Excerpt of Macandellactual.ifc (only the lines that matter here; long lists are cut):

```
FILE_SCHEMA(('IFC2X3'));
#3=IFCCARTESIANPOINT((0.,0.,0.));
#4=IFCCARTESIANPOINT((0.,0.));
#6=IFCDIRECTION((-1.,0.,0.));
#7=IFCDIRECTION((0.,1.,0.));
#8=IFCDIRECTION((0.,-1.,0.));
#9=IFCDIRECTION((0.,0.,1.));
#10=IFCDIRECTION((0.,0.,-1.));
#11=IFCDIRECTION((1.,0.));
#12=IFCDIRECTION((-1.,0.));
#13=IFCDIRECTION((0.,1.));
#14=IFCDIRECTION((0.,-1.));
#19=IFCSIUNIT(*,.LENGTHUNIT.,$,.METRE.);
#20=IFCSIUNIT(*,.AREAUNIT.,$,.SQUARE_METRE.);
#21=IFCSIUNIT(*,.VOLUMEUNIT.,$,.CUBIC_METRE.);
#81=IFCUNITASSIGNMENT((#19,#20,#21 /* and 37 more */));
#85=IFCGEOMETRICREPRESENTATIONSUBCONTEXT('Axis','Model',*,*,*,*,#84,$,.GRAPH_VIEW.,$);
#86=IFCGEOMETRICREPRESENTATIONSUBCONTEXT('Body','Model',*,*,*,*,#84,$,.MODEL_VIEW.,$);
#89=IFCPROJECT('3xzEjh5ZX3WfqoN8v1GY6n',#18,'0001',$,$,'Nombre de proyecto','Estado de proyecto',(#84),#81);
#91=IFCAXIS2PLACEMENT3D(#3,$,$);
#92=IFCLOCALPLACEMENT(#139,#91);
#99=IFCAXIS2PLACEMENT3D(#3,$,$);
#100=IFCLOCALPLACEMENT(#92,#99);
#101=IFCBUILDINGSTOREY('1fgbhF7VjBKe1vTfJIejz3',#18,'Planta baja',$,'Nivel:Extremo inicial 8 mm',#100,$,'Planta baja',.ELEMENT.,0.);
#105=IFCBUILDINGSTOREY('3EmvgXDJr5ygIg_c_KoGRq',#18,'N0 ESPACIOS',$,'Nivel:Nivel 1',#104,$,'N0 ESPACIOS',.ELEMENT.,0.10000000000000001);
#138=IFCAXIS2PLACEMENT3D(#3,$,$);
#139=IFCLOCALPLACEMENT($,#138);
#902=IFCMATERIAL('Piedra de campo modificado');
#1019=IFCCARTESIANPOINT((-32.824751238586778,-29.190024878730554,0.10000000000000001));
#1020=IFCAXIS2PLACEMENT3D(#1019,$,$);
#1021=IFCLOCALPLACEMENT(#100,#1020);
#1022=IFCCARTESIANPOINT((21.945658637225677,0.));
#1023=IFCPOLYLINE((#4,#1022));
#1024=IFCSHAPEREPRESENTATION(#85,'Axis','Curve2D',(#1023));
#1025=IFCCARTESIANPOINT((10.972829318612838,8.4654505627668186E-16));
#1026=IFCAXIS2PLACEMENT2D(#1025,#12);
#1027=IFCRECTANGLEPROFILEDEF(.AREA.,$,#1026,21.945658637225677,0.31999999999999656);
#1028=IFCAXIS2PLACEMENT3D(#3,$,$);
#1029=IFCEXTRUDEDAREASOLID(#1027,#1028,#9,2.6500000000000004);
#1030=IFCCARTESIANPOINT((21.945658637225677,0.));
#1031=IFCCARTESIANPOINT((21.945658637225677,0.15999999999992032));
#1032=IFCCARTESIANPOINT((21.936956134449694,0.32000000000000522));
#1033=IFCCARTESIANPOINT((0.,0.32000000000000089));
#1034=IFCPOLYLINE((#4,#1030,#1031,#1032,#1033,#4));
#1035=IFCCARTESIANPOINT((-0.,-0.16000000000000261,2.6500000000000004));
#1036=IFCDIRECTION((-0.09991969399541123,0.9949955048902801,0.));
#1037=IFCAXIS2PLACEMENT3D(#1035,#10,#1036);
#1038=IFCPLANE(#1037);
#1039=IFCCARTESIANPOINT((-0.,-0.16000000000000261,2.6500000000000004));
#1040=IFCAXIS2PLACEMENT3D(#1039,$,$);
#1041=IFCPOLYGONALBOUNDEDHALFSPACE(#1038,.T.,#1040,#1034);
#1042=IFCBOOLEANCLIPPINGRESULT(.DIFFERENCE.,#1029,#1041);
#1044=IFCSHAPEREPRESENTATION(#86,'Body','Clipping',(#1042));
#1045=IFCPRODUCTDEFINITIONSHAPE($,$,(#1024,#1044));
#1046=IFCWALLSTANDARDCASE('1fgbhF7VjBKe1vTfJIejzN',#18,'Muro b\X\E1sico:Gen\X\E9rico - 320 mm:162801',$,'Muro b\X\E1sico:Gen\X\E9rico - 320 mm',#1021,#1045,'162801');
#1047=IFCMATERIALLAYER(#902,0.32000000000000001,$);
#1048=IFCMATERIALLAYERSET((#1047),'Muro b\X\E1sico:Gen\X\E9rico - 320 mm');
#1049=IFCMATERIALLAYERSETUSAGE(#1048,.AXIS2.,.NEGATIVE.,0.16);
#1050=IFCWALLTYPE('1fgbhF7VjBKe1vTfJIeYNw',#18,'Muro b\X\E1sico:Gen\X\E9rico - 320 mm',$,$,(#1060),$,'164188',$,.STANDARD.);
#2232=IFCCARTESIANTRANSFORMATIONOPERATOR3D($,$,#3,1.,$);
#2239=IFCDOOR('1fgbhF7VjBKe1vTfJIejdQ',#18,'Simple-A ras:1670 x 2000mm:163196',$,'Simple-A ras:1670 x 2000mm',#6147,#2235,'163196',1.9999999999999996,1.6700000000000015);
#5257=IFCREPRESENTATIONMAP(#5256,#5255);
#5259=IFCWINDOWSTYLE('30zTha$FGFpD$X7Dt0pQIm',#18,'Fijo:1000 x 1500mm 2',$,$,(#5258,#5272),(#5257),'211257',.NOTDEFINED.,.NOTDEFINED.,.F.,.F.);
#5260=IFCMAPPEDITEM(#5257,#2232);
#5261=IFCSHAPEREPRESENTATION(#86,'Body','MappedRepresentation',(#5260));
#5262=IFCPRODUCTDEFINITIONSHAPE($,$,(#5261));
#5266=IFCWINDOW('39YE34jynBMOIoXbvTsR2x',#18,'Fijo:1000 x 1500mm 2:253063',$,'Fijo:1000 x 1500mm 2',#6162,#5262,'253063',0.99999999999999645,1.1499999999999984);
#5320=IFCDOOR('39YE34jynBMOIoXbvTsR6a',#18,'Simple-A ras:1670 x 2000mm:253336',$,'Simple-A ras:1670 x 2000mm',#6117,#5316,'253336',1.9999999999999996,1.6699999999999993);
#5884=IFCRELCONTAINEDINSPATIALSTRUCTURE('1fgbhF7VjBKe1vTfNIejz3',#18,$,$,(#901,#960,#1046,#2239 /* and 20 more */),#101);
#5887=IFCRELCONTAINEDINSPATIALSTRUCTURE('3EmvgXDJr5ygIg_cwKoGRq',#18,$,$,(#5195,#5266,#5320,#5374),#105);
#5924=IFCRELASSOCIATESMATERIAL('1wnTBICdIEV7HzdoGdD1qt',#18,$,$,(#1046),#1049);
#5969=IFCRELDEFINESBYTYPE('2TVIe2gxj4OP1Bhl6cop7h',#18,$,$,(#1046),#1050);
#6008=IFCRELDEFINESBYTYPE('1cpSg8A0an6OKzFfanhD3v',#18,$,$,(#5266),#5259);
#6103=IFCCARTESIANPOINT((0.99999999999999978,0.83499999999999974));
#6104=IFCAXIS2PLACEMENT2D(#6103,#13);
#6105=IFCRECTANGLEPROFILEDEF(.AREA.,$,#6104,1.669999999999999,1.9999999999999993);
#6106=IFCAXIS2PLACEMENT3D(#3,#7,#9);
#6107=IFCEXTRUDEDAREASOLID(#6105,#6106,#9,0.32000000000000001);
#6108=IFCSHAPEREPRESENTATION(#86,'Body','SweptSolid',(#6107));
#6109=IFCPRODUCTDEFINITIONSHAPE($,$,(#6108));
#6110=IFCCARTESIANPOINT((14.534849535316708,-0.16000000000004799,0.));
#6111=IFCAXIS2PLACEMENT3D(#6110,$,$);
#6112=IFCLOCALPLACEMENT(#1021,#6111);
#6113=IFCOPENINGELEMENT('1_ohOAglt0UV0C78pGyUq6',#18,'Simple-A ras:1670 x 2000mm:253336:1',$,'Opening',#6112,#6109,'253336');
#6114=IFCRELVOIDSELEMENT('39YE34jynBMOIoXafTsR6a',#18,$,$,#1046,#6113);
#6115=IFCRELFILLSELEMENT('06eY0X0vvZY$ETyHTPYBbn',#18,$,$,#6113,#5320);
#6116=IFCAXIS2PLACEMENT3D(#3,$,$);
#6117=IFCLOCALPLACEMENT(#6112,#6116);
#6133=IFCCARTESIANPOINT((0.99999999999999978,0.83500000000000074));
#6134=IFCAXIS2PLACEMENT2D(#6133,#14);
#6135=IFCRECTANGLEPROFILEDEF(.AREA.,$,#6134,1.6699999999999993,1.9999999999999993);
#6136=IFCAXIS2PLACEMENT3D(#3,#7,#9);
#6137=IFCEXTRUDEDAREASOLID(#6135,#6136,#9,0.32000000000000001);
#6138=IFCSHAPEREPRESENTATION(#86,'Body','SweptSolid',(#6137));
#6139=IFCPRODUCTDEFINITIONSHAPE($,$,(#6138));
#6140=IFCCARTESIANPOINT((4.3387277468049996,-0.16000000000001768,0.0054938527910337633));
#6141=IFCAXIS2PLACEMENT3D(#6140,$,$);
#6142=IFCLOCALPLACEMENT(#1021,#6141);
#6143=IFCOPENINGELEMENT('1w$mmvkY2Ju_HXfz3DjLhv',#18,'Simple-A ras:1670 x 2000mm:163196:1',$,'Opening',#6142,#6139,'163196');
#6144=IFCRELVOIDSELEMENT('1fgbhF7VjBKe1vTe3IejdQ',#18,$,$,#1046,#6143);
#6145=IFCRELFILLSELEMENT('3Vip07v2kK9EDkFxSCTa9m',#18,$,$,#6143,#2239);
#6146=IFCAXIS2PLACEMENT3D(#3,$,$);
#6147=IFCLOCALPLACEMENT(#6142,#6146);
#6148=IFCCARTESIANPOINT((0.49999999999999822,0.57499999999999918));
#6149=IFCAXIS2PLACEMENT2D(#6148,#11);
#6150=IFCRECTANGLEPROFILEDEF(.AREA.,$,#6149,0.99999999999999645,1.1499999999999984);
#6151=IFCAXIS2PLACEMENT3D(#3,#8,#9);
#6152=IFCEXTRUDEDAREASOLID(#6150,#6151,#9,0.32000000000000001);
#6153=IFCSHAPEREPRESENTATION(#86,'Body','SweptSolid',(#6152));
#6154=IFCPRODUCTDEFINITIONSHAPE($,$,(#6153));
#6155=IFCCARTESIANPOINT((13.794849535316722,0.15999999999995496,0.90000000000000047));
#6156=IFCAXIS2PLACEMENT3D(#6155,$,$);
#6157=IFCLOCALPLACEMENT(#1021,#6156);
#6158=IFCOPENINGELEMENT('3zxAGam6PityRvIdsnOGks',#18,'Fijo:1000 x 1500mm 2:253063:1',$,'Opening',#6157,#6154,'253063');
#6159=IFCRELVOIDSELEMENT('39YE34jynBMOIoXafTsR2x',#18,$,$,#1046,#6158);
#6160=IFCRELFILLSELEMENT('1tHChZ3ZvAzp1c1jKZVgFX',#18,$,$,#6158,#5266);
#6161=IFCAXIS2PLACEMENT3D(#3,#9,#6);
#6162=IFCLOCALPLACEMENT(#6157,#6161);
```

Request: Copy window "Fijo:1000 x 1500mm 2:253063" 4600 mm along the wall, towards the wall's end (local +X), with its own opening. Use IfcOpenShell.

```python
import ifcopenshell
import ifcopenshell.api.feature
import ifcopenshell.api.geometry
import ifcopenshell.api.root
import ifcopenshell.geom
import ifcopenshell.util.element
import ifcopenshell.util.placement
import ifcopenshell.util.shape
import ifcopenshell.util.unit

model = ifcopenshell.open("Macandellactual.ifc")
unit_scale = ifcopenshell.util.unit.calculate_unit_scale(model)
settings = ifcopenshell.geom.settings()


def volume(element):
    """Net volume in cubic metres, openings subtracted."""
    shape = ifcopenshell.geom.create_shape(settings, element)
    return ifcopenshell.util.shape.get_volume(shape.geometry)


def reuse_history(source, copy):
    """copy_class also copies each property set's owner history, people and application; keep the originals."""
    for rel in copy.IsDefinedBy:
        if rel.is_a("IfcRelDefinesByProperties") and (history := rel.RelatingPropertyDefinition.OwnerHistory):
            rel.RelatingPropertyDefinition.OwnerHistory = source.OwnerHistory
            ifcopenshell.util.element.remove_deep2(model, history)


window = model.by_guid("39YE34jynBMOIoXbvTsR2x")
opening = window.FillsVoids[0].RelatingOpeningElement
wall = opening.VoidsElements[0].RelatingBuildingElement
before = volume(wall)
shift = ifcopenshell.util.placement.get_local_placement(wall.ObjectPlacement)[:3, 0] * 4.6 / unit_scale

# copy_class copies the void relationship, type, container and properties, but no geometry.
new_opening = ifcopenshell.api.root.copy_class(model, product=opening)
new_opening.Representation = ifcopenshell.util.element.copy_deep(
    model, opening.Representation, exclude=["IfcGeometricRepresentationContext", "IfcRepresentationMap"]
)
new_opening.Name = "Fijo:1000 x 1500mm 2"
new_opening.Tag = None
new_window = ifcopenshell.api.root.copy_class(model, product=window)
new_window.Representation = ifcopenshell.util.element.copy_deep(
    model, window.Representation, exclude=["IfcGeometricRepresentationContext", "IfcRepresentationMap"]
)
new_window.Name = "Fijo:1000 x 1500mm 2"
new_window.Tag = None
reuse_history(window, new_window)
fills = ifcopenshell.api.feature.add_filling(model, opening=new_opening, element=new_window)
fills.OwnerHistory = new_window.OwnerHistory  # required in IFC2X3

for old, new in ((opening, new_opening), (window, new_window)):
    matrix = ifcopenshell.util.placement.get_local_placement(old.ObjectPlacement)
    matrix[:3, 3] += shift
    ifcopenshell.api.geometry.edit_object_placement(model, product=new, matrix=matrix, is_si=False)

after = volume(wall)

print(f"wall volume {before:.3f} -> {after:.3f} m3")

model.write("Macandellactual-out.ifc")
```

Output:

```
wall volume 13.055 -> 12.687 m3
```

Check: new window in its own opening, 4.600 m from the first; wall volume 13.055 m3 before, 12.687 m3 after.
